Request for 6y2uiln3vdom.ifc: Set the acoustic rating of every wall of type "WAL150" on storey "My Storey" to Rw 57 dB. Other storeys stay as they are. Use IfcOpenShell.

First a look at what the model holds.

```python
import ifcopenshell
import ifcopenshell.util.element

model = ifcopenshell.open("6y2uiln3vdom.ifc")
print(model.schema)
storey = next(s for s in model.by_type("IfcBuildingStorey") if s.Name == "My Storey")
walls = [e for e in ifcopenshell.util.element.get_decomposition(storey) if e.is_a("IfcWall")]
seen = {}
for e in walls:
    element_type = ifcopenshell.util.element.get_type(e)
    key = (element_type.Name if element_type != e and element_type else None, ifcopenshell.util.element.get_pset(e, "Pset_WallCommon", "AcousticRating"))
    seen[key] = seen.get(key, 0) + 1
for (name, value), count in sorted(seen.items(), key=str):
    print(count, "x", name, "|", value)
```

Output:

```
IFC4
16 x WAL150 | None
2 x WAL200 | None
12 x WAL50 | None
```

```python
import ifcopenshell
import ifcopenshell.api.pset
import ifcopenshell.util.element

model = ifcopenshell.open("6y2uiln3vdom.ifc")

storey = next(s for s in model.by_type("IfcBuildingStorey") if s.Name == "My Storey")
walls = [e for e in ifcopenshell.util.element.get_decomposition(storey) if e.is_a("IfcWall")]

count = 0
for e in walls:
    element_type = ifcopenshell.util.element.get_type(e)
    if element_type in (None, e) or element_type.Name != "WAL150":
        continue
    # add_pset returns the element's existing set when there is one.
    pset = ifcopenshell.api.pset.add_pset(model, product=e, name="Pset_WallCommon")
    ifcopenshell.api.pset.edit_pset(model, pset=pset, properties={"AcousticRating": "Rw 57 dB"})
    count += 1

print(count, "walls updated")

model.write("6y2uiln3vdom-out.ifc")
```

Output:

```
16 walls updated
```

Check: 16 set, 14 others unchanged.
